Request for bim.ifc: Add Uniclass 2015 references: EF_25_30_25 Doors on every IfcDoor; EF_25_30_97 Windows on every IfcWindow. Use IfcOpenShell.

First a look at what the model holds.

```python
import ifcopenshell

model = ifcopenshell.open("bim.ifc")
print(model.schema)
print("classifications:", [c.Name for c in model.by_type("IfcClassification")])
for ifc_class in ("IfcDoor", "IfcRoof", "IfcStair", "IfcWall", "IfcWindow"):
    print(ifc_class, len(model.by_type(ifc_class)))
```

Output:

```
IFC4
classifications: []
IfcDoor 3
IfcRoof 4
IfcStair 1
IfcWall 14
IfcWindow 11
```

```python
import ifcopenshell
import ifcopenshell.api.classification

model = ifcopenshell.open("bim.ifc")

system = ifcopenshell.api.classification.add_classification(model, classification="Uniclass 2015")

codes = {
    "IfcDoor": ("EF_25_30_25", "Doors"),
    "IfcWindow": ("EF_25_30_97", "Windows"),
}
for ifc_class, (code, name) in codes.items():
    products = model.by_type(ifc_class)
    ifcopenshell.api.classification.add_reference(
        model, products=products, classification=system, identification=code, name=name
    )
    print(code, len(products))

model.write("bim_rev.ifc")
```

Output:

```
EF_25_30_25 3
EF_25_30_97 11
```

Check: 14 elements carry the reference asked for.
